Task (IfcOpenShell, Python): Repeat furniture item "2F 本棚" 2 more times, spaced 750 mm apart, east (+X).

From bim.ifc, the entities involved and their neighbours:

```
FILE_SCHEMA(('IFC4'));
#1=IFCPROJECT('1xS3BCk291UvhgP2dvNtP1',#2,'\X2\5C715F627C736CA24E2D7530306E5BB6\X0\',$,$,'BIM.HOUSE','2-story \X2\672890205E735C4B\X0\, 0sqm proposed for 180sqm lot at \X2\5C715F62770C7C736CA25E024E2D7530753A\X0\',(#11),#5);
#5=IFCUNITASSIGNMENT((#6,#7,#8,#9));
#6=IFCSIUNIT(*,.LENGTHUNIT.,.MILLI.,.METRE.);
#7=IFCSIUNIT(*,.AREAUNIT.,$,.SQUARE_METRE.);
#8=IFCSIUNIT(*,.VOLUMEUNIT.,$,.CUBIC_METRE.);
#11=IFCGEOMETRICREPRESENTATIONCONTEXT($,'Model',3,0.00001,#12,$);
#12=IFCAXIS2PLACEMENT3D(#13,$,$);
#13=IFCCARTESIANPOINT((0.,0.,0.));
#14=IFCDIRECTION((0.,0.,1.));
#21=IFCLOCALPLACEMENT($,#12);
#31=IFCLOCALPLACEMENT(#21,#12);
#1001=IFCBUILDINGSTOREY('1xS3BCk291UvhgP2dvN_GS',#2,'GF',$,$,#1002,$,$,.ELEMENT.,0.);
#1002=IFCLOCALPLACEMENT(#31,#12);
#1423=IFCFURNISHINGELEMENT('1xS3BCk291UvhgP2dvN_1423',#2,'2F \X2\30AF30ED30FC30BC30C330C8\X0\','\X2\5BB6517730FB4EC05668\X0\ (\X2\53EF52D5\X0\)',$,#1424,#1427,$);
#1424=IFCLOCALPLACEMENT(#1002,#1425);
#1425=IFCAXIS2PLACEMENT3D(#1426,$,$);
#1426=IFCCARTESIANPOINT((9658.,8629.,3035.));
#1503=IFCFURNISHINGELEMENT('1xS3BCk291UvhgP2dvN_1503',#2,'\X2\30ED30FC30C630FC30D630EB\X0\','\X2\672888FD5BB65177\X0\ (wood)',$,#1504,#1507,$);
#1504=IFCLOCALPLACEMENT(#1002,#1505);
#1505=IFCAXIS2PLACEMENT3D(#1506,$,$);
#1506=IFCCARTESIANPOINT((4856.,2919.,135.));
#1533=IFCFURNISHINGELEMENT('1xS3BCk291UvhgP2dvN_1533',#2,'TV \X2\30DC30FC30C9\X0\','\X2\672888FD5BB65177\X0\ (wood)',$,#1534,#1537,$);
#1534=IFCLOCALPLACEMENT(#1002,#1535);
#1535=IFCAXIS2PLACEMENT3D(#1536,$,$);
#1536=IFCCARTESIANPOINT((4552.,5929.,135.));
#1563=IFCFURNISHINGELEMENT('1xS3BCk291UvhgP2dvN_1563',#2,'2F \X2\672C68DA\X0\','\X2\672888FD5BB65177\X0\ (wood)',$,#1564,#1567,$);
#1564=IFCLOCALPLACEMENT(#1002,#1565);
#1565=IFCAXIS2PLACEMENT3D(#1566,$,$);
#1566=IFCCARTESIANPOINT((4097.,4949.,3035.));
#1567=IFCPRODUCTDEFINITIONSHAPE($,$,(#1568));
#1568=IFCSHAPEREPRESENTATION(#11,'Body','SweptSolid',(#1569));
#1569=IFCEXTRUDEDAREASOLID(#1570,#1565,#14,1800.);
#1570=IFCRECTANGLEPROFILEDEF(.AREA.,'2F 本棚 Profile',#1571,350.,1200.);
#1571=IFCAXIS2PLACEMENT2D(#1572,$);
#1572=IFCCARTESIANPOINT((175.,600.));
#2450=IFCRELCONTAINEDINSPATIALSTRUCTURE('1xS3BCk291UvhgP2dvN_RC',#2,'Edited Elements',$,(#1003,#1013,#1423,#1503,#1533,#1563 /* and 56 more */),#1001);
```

```python
import numpy as np
import ifcopenshell
import ifcopenshell.api.geometry
import ifcopenshell.api.root
import ifcopenshell.util.element
import ifcopenshell.util.placement
import ifcopenshell.util.unit

model = ifcopenshell.open("bim.ifc")
unit_scale = ifcopenshell.util.unit.calculate_unit_scale(model)


def reuse_history(source, copy):
    """copy_class also copies each property set's owner history, people and application; keep the originals."""
    for rel in copy.IsDefinedBy:
        if rel.is_a("IfcRelDefinesByProperties") and (history := rel.RelatingPropertyDefinition.OwnerHistory):
            rel.RelatingPropertyDefinition.OwnerHistory = source.OwnerHistory
            ifcopenshell.util.element.remove_deep2(model, history)


source = model.by_guid("1xS3BCk291UvhgP2dvN_1563")
base = ifcopenshell.util.placement.get_local_placement(source.ObjectPlacement)
step = np.array([1.0, 0.0, 0.0]) * 0.75 / unit_scale

for i in range(1, 3):
    copy = ifcopenshell.api.root.copy_class(model, product=source)
    copy.Representation = ifcopenshell.util.element.copy_deep(
        model, source.Representation, exclude=["IfcGeometricRepresentationContext", "IfcRepresentationMap"]
    )
    reuse_history(source, copy)
    matrix = base.copy()
    matrix[:3, 3] += i * step
    print("added at", matrix[:3, 3].round(3) + 0.0)
    ifcopenshell.api.geometry.edit_object_placement(model, product=copy, matrix=matrix, is_si=False)

model.write("bim_edited.ifc")
```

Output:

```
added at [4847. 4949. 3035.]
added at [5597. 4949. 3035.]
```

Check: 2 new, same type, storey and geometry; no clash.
